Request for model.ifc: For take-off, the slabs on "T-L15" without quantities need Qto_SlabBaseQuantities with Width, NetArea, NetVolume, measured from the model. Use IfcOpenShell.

First a look at what the model holds.

```python
import ifcopenshell
import ifcopenshell.util.element
import ifcopenshell.util.unit

model = ifcopenshell.open("model.ifc")
print(model.schema)
for unit_type in ("LENGTHUNIT", "AREAUNIT", "VOLUMEUNIT"):
    print(unit_type, ifcopenshell.util.unit.calculate_unit_scale(model, unit_type))
storey = next(s for s in model.by_type("IfcBuildingStorey") if s.Name == "T-L15")
slabs = [e for e in ifcopenshell.util.element.get_decomposition(storey) if e.is_a("IfcSlab")]
for e in sorted(slabs, key=lambda e: e.id()):
    print(e.id(), e.is_a(), e.Name, list(ifcopenshell.util.element.get_psets(e, qtos_only=True)), sep=" | ")
```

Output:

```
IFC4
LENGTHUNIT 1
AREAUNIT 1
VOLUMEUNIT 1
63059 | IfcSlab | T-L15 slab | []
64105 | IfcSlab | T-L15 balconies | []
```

```python
import ifcopenshell
import ifcopenshell.api.pset
import ifcopenshell.geom
import ifcopenshell.util.element
import ifcopenshell.util.shape
import ifcopenshell.util.unit

model = ifcopenshell.open("model.ifc")
unit_scale = ifcopenshell.util.unit.calculate_unit_scale(model)
area_scale = ifcopenshell.util.unit.calculate_unit_scale(model, "AREAUNIT")
volume_scale = ifcopenshell.util.unit.calculate_unit_scale(model, "VOLUMEUNIT")
settings = ifcopenshell.geom.settings()

storey = next(s for s in model.by_type("IfcBuildingStorey") if s.Name == "T-L15")
slabs = [e for e in ifcopenshell.util.element.get_decomposition(storey) if e.is_a("IfcSlab")]

for e in sorted(slabs, key=lambda e: e.id()):
    if ifcopenshell.util.element.get_psets(e, qtos_only=True, should_inherit=False):
        continue
    # Geometry comes back in metres, in the element's own axes.
    shape = ifcopenshell.geom.create_shape(settings, e)
    values = {
        "Width": ifcopenshell.util.shape.get_z(shape.geometry) / unit_scale,
        "NetArea": ifcopenshell.util.shape.get_footprint_area(shape.geometry) / area_scale,
        "NetVolume": ifcopenshell.util.shape.get_volume(shape.geometry) / volume_scale,
    }
    qto = ifcopenshell.api.pset.add_qto(model, product=e, name="Qto_SlabBaseQuantities")
    ifcopenshell.api.pset.edit_qto(model, qto=qto, properties=values)
    print(e.id(), {k: round(v, 3) for k, v in values.items()})

model.write("model_updated.ifc")
```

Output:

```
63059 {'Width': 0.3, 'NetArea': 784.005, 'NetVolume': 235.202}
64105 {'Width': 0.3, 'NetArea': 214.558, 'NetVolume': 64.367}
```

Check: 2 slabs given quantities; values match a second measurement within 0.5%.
